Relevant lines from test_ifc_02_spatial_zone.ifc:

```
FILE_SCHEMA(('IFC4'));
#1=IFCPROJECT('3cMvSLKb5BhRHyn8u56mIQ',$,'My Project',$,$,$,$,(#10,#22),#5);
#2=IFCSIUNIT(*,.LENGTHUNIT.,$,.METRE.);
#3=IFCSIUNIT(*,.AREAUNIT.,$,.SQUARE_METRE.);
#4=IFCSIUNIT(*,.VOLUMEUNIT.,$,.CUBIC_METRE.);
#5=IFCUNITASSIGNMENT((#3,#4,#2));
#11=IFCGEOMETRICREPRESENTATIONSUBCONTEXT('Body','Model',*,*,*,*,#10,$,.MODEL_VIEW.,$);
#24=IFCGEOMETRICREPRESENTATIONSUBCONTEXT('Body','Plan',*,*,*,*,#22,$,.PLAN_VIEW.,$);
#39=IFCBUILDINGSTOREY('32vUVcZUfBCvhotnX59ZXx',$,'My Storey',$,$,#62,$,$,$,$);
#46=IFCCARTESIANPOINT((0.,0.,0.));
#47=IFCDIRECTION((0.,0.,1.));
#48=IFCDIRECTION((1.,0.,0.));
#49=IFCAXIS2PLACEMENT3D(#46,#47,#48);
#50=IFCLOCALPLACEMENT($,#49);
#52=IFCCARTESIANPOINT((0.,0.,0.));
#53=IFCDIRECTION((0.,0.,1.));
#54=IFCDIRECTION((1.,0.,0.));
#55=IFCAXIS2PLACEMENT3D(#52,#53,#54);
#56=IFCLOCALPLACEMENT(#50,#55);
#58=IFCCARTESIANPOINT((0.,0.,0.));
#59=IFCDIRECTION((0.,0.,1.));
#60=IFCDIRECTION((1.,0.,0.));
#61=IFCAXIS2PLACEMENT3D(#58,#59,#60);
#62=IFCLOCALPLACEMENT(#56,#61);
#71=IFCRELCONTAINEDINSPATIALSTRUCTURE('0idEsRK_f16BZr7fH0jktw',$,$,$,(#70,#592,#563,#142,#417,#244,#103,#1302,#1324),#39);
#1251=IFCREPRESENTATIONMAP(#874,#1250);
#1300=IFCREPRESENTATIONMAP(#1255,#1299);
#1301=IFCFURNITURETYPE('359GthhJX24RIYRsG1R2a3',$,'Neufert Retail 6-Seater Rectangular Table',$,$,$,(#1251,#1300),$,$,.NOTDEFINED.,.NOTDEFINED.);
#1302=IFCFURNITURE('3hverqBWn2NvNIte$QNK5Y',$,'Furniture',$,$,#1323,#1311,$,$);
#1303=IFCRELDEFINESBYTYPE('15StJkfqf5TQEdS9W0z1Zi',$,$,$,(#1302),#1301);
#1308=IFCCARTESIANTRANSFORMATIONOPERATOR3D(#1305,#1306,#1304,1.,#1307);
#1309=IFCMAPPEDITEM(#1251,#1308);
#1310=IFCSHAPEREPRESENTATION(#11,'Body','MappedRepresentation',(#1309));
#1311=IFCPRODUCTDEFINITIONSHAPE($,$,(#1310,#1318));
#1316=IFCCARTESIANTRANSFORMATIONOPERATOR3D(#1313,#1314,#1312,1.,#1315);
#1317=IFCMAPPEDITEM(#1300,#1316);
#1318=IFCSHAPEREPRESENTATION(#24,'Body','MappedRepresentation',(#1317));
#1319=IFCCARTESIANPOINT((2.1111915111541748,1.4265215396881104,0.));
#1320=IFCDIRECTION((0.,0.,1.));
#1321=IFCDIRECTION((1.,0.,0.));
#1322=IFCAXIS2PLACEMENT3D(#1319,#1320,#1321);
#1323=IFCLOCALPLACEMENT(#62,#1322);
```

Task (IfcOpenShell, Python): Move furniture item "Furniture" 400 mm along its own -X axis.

```python
import ifcopenshell
import ifcopenshell.api.geometry
import ifcopenshell.util.placement
import ifcopenshell.util.unit

model = ifcopenshell.open("test_ifc_02_spatial_zone.ifc")
unit_scale = ifcopenshell.util.unit.calculate_unit_scale(model)

item = model.by_id(1302)
matrix = ifcopenshell.util.placement.get_local_placement(item.ObjectPlacement)
matrix[:3, 3] -= matrix[:3, 0] * 0.4 / unit_scale
ifcopenshell.api.geometry.edit_object_placement(model, product=item, matrix=matrix, is_si=False)

print(ifcopenshell.util.placement.get_local_placement(item.ObjectPlacement).round(3) + 0.0)

model.write("test_ifc_02_spatial_zone_edited.ifc")
```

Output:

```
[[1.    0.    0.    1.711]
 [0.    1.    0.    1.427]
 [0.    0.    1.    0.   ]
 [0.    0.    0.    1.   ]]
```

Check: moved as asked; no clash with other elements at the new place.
